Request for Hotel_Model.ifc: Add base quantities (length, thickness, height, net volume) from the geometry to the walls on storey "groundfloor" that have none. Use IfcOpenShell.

First a look at what the model holds.

```python
import ifcopenshell
import ifcopenshell.util.element
import ifcopenshell.util.unit

model = ifcopenshell.open("Hotel_Model.ifc")
print(model.schema)
for unit_type in ("LENGTHUNIT", "AREAUNIT", "VOLUMEUNIT"):
    print(unit_type, ifcopenshell.util.unit.calculate_unit_scale(model, unit_type))
storey = next(s for s in model.by_type("IfcBuildingStorey") if s.Name == "groundfloor")
walls = [e for e in ifcopenshell.util.element.get_decomposition(storey) if e.is_a("IfcWall")]
for e in sorted(walls, key=lambda e: e.id()):
    print(e.id(), e.is_a(), e.Name, list(ifcopenshell.util.element.get_psets(e, qtos_only=True)), sep=" | ")
```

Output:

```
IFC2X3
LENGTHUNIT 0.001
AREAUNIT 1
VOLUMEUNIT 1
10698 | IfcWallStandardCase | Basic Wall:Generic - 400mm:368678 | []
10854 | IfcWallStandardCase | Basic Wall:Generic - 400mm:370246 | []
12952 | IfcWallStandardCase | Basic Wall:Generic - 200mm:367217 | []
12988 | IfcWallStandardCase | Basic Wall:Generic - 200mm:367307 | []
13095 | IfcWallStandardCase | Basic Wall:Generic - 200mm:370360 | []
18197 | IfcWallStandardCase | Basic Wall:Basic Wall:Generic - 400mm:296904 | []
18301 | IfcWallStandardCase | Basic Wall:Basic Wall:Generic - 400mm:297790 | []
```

```python
import ifcopenshell
import ifcopenshell.api.pset
import ifcopenshell.geom
import ifcopenshell.util.element
import ifcopenshell.util.shape
import ifcopenshell.util.unit

model = ifcopenshell.open("Hotel_Model.ifc")
unit_scale = ifcopenshell.util.unit.calculate_unit_scale(model)
volume_scale = ifcopenshell.util.unit.calculate_unit_scale(model, "VOLUMEUNIT")
settings = ifcopenshell.geom.settings()

storey = next(s for s in model.by_type("IfcBuildingStorey") if s.Name == "groundfloor")
walls = [e for e in ifcopenshell.util.element.get_decomposition(storey) if e.is_a("IfcWall")]

for e in sorted(walls, key=lambda e: e.id()):
    if ifcopenshell.util.element.get_psets(e, qtos_only=True, should_inherit=False):
        continue
    # Geometry comes back in metres, in the element's own axes.
    shape = ifcopenshell.geom.create_shape(settings, e)
    values = {
        "Length": ifcopenshell.util.shape.get_x(shape.geometry) / unit_scale,
        "Width": ifcopenshell.util.shape.get_y(shape.geometry) / unit_scale,
        "Height": ifcopenshell.util.shape.get_z(shape.geometry) / unit_scale,
        "NetVolume": ifcopenshell.util.shape.get_volume(shape.geometry) / volume_scale,
    }
    qto = ifcopenshell.api.pset.add_qto(model, product=e, name="BaseQuantities")
    ifcopenshell.api.pset.edit_qto(model, qto=qto, properties=values)
    print(e.id(), {k: round(v, 3) for k, v in values.items()})

model.write("Hotel_Model_updated.ifc")
```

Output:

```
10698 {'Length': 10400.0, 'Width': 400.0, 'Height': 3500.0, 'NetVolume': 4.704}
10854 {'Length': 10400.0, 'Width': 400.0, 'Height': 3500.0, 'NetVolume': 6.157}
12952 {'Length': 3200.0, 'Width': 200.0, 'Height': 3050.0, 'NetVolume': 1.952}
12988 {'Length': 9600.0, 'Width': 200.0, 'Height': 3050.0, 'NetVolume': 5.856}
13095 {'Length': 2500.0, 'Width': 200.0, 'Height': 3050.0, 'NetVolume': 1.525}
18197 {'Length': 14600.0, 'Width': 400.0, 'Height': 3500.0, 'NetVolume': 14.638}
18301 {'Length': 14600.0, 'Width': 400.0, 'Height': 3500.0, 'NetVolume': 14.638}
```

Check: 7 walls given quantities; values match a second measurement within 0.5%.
